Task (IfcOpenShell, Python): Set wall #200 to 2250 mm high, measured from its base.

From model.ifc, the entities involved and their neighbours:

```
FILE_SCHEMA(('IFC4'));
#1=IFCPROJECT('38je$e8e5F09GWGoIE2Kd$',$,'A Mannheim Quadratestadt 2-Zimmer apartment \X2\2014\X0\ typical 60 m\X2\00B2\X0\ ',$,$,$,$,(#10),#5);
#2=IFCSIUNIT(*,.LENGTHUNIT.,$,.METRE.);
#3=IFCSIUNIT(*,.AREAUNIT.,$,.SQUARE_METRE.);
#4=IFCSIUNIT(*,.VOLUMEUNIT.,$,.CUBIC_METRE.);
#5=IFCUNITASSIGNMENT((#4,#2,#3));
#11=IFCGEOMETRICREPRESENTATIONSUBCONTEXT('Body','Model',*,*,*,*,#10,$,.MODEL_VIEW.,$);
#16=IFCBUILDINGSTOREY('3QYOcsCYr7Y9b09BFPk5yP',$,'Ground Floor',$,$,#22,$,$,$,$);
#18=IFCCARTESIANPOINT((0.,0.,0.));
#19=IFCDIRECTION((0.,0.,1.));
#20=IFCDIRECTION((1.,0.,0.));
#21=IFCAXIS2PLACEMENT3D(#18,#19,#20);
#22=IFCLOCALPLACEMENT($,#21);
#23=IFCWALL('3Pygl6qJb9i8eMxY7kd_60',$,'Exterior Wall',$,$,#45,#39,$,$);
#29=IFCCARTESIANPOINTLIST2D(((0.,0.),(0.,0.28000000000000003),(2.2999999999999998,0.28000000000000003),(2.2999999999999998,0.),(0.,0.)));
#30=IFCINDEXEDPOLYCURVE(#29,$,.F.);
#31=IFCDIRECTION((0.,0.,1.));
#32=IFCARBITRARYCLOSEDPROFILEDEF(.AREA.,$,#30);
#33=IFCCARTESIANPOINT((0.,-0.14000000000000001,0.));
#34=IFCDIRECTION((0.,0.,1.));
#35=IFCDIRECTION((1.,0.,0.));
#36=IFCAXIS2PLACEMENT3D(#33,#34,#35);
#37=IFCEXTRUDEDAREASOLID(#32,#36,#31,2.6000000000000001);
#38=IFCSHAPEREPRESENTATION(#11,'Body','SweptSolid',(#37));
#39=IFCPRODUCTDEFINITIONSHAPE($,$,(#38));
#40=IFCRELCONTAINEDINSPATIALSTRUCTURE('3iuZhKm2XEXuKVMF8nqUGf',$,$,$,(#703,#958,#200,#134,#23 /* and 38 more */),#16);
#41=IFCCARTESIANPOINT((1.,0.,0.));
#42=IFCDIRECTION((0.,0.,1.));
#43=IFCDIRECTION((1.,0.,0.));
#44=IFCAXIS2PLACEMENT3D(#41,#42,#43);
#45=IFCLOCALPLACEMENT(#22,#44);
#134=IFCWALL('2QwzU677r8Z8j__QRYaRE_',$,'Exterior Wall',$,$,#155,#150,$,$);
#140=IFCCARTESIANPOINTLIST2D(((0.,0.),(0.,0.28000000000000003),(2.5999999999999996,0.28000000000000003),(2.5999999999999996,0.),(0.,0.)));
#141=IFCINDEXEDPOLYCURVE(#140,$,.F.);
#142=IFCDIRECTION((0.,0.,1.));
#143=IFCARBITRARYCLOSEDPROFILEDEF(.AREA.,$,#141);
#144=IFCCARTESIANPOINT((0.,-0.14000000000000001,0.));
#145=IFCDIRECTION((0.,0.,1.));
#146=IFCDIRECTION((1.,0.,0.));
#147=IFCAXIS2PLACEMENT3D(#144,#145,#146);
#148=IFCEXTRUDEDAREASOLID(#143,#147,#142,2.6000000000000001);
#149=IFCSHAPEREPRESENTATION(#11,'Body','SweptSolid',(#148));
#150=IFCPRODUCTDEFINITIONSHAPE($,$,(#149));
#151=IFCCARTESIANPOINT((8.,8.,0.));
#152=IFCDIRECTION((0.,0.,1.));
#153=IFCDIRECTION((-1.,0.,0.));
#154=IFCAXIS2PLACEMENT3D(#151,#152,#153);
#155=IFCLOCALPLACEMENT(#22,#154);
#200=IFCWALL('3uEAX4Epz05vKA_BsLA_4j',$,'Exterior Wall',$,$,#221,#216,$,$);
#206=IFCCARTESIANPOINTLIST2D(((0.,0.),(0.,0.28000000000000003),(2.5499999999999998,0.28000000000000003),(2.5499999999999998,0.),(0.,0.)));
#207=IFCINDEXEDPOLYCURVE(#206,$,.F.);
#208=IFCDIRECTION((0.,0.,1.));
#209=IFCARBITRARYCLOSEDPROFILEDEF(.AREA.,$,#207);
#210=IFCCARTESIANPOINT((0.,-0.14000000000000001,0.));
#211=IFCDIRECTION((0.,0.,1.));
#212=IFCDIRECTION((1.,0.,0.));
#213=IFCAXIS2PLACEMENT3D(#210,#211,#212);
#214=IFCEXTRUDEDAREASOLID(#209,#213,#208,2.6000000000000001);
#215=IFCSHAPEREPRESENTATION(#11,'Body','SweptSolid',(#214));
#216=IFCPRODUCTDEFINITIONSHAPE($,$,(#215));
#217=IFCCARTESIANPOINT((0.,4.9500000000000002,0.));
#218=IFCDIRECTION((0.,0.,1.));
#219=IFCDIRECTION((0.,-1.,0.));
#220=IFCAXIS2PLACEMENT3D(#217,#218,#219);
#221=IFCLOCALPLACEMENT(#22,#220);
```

```python
import ifcopenshell
import ifcopenshell.geom
import ifcopenshell.util.representation
import ifcopenshell.util.shape
import ifcopenshell.util.unit

model = ifcopenshell.open("model.ifc")
unit_scale = ifcopenshell.util.unit.calculate_unit_scale(model)
settings = ifcopenshell.geom.settings()


def volume(element):
    """Net volume in cubic metres, openings subtracted."""
    shape = ifcopenshell.geom.create_shape(settings, element)
    return ifcopenshell.util.shape.get_volume(shape.geometry)


wall = model.by_guid("3uEAX4Epz05vKA_BsLA_4j")
before = volume(wall)

body = ifcopenshell.util.representation.get_representation(wall, "Model", "Body")
solid = body.Items[0]
old_height = solid.Depth
solid.Depth = 2.25 / unit_scale
after = volume(wall)

print(f"height {old_height:g} -> {solid.Depth:g}, volume {before:.3f} -> {after:.3f} m3")

model.write("model_edited.ifc")
```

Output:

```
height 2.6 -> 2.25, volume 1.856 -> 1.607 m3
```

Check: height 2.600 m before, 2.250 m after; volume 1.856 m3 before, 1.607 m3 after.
